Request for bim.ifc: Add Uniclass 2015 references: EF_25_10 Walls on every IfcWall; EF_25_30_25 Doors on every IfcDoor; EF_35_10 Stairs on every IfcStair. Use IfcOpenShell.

First a look at what the model holds.

```python
import ifcopenshell

model = ifcopenshell.open("bim.ifc")
print(model.schema)
print("classifications:", [c.Name for c in model.by_type("IfcClassification")])
for ifc_class in ("IfcDoor", "IfcRoof", "IfcStair", "IfcWall", "IfcWindow"):
    print(ifc_class, len(model.by_type(ifc_class)))
```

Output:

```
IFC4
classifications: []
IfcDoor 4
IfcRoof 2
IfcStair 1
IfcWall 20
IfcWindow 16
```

```python
import ifcopenshell
import ifcopenshell.api.classification

model = ifcopenshell.open("bim.ifc")

system = ifcopenshell.api.classification.add_classification(model, classification="Uniclass 2015")

codes = {
    "IfcWall": ("EF_25_10", "Walls"),
    "IfcDoor": ("EF_25_30_25", "Doors"),
    "IfcStair": ("EF_35_10", "Stairs"),
}
for ifc_class, (code, name) in codes.items():
    products = model.by_type(ifc_class)
    ifcopenshell.api.classification.add_reference(
        model, products=products, classification=system, identification=code, name=name
    )
    print(code, len(products))

model.write("bim_updated.ifc")
```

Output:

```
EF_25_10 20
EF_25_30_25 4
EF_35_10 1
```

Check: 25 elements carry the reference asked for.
